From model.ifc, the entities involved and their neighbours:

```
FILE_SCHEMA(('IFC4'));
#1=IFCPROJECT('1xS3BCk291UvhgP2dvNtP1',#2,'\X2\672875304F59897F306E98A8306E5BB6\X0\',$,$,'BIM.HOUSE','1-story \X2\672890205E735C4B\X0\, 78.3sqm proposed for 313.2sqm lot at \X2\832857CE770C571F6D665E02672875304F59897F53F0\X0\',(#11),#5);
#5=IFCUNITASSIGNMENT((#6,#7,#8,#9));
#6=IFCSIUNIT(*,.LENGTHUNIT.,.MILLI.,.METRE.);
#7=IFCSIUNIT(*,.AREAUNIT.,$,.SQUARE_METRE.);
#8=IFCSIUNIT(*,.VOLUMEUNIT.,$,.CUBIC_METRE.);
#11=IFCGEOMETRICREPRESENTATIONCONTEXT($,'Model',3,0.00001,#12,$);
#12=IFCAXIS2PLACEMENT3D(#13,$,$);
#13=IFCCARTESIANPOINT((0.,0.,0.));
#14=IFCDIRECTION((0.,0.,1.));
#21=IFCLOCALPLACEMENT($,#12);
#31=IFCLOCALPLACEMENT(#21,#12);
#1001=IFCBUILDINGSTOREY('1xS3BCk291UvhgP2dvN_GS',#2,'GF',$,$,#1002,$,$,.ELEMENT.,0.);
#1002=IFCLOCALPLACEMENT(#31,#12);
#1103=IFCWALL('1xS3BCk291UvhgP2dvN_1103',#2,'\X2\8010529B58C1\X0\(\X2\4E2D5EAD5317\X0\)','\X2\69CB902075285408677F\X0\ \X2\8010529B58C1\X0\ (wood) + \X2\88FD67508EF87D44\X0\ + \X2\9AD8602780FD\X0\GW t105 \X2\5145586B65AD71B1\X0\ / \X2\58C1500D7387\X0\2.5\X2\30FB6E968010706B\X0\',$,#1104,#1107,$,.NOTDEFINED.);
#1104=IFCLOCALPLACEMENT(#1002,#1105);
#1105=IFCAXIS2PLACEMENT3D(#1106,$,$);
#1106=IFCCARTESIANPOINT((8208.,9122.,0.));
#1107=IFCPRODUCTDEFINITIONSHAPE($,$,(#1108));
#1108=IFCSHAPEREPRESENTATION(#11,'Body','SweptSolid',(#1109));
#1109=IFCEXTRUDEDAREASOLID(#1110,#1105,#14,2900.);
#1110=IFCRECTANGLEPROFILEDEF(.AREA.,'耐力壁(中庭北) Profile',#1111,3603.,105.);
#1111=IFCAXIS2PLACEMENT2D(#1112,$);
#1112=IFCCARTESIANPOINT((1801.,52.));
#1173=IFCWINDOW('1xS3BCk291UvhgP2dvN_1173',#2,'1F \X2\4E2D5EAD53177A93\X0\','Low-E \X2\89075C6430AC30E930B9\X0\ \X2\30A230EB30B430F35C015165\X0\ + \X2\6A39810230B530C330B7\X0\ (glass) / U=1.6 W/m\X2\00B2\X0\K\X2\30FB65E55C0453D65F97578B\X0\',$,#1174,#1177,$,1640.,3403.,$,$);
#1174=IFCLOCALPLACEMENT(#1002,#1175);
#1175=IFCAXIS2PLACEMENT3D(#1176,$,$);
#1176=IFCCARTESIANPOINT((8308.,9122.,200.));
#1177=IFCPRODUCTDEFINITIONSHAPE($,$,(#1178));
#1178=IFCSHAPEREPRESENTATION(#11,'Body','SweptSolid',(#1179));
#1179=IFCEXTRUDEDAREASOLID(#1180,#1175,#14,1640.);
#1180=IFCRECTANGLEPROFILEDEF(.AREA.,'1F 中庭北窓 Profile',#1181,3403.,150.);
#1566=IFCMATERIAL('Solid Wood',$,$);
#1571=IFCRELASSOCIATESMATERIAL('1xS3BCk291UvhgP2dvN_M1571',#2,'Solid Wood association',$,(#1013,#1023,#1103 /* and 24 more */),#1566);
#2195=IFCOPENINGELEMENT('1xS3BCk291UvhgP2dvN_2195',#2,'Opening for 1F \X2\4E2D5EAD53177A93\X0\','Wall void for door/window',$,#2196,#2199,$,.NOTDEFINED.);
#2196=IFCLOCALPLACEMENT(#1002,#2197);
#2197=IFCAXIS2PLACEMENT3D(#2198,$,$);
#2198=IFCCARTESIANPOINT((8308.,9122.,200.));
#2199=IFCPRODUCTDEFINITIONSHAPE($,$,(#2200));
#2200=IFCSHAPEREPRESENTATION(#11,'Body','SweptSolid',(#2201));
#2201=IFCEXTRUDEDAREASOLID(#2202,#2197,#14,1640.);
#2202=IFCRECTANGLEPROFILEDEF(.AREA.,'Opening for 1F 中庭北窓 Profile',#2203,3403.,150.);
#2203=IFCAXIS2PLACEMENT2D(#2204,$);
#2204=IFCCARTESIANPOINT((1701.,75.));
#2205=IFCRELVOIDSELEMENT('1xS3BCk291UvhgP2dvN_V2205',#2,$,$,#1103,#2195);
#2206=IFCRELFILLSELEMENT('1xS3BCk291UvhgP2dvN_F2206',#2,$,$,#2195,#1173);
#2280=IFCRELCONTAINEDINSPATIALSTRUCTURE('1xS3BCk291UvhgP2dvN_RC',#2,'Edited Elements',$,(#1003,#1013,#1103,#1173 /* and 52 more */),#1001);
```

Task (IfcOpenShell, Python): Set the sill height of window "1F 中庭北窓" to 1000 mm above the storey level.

```python
import numpy as np
import ifcopenshell
import ifcopenshell.api.geometry
import ifcopenshell.geom
import ifcopenshell.util.element
import ifcopenshell.util.placement
import ifcopenshell.util.shape
import ifcopenshell.util.unit

model = ifcopenshell.open("model.ifc")
unit_scale = ifcopenshell.util.unit.calculate_unit_scale(model)

window = model.by_id(1173)
opening = window.FillsVoids[0].RelatingOpeningElement
storey = ifcopenshell.util.element.get_container(window, ifc_class="IfcBuildingStorey")
level = ifcopenshell.util.placement.get_local_placement(storey.ObjectPlacement)[2, 3]

# The opening's origin need not be at the sill, so measure its lowest point.
shape = ifcopenshell.geom.create_shape(ifcopenshell.geom.settings(), opening)
bottom = ifcopenshell.util.shape.get_shape_bottom_elevation(shape, shape.geometry) / unit_scale
dz = level + 1000.0 - bottom

shift = np.array([0.0, 0.0, dz])
# The window is not placed relative to its opening, so move both.
for product in (opening, window):
    matrix = ifcopenshell.util.placement.get_local_placement(product.ObjectPlacement)
    matrix[:3, 3] += shift
    ifcopenshell.api.geometry.edit_object_placement(model, product=product, matrix=matrix, is_si=False)

print(f"moved by {dz * unit_scale:+.3f} m")

model.write("model-out.ifc")
```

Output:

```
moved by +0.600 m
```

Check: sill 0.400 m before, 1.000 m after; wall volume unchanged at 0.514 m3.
